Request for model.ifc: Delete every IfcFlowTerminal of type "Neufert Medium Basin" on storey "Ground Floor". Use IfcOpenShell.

First a look at what the model holds.

```python
import ifcopenshell
import ifcopenshell.util.element

model = ifcopenshell.open("model.ifc")
print(model.schema)
storey = next(s for s in model.by_type("IfcBuildingStorey") if s.Name == "Ground Floor")
terminals = [e for e in ifcopenshell.util.element.get_decomposition(storey) if e.is_a("IfcFlowTerminal")]
seen = {}
for e in terminals:
    element_type = ifcopenshell.util.element.get_type(e)
    name = element_type.Name if element_type not in (None, e) else None
    seen[name] = seen.get(name, 0) + 1
for name, count in sorted(seen.items(), key=str):
    print(count, "x", name)
```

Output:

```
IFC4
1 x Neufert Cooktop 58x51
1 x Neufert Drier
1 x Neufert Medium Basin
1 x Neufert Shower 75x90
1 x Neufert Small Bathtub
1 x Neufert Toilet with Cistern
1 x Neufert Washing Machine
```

```python
import ifcopenshell
import ifcopenshell.api.root
import ifcopenshell.util.element

model = ifcopenshell.open("model.ifc")

storey = next(s for s in model.by_type("IfcBuildingStorey") if s.Name == "Ground Floor")
terminals = [e for e in ifcopenshell.util.element.get_decomposition(storey) if e.is_a("IfcFlowTerminal")]
targets = [e for e in terminals if (t := ifcopenshell.util.element.get_type(e)) not in (None, e) and t.Name == "Neufert Medium Basin"]

for e in targets:
    ifcopenshell.api.root.remove_product(model, product=e)
print(len(targets), "removed")

model.write("model_edited.ifc")
```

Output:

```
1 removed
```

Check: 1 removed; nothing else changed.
